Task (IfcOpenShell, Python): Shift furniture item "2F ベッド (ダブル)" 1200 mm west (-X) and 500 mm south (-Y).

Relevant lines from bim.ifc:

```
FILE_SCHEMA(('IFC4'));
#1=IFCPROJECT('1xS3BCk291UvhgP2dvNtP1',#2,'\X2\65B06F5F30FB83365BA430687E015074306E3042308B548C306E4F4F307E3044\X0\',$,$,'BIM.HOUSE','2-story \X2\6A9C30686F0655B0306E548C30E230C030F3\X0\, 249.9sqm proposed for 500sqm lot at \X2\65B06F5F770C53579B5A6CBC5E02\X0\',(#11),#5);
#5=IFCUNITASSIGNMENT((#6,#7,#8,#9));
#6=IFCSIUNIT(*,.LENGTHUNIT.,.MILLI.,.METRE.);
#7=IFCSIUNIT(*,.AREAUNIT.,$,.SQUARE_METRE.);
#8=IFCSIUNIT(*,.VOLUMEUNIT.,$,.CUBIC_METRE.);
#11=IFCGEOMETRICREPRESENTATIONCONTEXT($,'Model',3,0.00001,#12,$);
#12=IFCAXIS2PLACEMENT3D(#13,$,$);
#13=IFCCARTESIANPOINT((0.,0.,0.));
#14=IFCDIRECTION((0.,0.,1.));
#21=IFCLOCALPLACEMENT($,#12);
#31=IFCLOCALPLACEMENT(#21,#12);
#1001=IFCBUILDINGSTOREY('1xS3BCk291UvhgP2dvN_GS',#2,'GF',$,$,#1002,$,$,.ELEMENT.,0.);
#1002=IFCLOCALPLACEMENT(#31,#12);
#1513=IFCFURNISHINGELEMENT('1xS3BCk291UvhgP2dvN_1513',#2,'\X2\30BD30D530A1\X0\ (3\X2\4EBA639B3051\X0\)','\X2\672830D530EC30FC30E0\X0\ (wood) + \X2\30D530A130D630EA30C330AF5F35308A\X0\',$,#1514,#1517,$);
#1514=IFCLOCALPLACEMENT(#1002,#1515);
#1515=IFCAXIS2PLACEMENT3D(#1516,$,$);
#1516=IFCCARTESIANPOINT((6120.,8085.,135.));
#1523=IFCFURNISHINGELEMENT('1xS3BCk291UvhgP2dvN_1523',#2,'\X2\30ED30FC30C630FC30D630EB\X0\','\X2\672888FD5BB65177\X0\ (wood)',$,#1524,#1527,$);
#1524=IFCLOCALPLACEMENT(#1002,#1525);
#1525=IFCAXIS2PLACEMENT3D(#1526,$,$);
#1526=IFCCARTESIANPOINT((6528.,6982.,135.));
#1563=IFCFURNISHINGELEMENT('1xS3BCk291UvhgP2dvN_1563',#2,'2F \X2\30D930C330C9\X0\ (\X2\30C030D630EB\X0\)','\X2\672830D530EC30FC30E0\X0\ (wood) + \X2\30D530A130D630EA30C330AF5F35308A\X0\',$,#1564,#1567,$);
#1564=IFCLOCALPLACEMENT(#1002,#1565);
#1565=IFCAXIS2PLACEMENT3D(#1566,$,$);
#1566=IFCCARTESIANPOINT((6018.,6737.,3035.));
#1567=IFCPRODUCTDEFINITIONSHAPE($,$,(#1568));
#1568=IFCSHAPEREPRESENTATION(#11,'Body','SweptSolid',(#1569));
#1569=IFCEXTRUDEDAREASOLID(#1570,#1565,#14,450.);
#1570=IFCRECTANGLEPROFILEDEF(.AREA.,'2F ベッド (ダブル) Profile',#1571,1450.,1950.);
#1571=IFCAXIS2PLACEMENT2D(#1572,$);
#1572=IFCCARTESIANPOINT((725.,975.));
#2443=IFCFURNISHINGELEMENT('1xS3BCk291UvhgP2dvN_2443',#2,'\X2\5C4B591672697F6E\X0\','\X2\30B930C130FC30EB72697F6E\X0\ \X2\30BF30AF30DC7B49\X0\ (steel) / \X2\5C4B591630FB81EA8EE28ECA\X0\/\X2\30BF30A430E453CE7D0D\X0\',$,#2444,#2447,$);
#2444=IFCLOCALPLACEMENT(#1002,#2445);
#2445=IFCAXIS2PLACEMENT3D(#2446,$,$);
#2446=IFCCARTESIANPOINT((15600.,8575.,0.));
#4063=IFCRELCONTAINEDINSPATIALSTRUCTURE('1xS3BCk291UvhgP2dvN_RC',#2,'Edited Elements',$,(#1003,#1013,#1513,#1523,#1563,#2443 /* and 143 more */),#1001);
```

```python
import ifcopenshell
import ifcopenshell.api.geometry
import ifcopenshell.util.placement
import ifcopenshell.util.unit

model = ifcopenshell.open("bim.ifc")
unit_scale = ifcopenshell.util.unit.calculate_unit_scale(model)

item = model.by_id(1563)
matrix = ifcopenshell.util.placement.get_local_placement(item.ObjectPlacement)
matrix[0, 3] -= 1.2 / unit_scale
matrix[1, 3] -= 0.5 / unit_scale
ifcopenshell.api.geometry.edit_object_placement(model, product=item, matrix=matrix, is_si=False)

print(ifcopenshell.util.placement.get_local_placement(item.ObjectPlacement).round(3) + 0.0)

model.write("bim_updated.ifc")
```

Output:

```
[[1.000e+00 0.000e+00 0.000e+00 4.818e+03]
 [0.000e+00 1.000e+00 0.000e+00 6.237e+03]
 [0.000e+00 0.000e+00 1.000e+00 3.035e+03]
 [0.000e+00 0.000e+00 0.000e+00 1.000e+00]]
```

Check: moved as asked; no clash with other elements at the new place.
